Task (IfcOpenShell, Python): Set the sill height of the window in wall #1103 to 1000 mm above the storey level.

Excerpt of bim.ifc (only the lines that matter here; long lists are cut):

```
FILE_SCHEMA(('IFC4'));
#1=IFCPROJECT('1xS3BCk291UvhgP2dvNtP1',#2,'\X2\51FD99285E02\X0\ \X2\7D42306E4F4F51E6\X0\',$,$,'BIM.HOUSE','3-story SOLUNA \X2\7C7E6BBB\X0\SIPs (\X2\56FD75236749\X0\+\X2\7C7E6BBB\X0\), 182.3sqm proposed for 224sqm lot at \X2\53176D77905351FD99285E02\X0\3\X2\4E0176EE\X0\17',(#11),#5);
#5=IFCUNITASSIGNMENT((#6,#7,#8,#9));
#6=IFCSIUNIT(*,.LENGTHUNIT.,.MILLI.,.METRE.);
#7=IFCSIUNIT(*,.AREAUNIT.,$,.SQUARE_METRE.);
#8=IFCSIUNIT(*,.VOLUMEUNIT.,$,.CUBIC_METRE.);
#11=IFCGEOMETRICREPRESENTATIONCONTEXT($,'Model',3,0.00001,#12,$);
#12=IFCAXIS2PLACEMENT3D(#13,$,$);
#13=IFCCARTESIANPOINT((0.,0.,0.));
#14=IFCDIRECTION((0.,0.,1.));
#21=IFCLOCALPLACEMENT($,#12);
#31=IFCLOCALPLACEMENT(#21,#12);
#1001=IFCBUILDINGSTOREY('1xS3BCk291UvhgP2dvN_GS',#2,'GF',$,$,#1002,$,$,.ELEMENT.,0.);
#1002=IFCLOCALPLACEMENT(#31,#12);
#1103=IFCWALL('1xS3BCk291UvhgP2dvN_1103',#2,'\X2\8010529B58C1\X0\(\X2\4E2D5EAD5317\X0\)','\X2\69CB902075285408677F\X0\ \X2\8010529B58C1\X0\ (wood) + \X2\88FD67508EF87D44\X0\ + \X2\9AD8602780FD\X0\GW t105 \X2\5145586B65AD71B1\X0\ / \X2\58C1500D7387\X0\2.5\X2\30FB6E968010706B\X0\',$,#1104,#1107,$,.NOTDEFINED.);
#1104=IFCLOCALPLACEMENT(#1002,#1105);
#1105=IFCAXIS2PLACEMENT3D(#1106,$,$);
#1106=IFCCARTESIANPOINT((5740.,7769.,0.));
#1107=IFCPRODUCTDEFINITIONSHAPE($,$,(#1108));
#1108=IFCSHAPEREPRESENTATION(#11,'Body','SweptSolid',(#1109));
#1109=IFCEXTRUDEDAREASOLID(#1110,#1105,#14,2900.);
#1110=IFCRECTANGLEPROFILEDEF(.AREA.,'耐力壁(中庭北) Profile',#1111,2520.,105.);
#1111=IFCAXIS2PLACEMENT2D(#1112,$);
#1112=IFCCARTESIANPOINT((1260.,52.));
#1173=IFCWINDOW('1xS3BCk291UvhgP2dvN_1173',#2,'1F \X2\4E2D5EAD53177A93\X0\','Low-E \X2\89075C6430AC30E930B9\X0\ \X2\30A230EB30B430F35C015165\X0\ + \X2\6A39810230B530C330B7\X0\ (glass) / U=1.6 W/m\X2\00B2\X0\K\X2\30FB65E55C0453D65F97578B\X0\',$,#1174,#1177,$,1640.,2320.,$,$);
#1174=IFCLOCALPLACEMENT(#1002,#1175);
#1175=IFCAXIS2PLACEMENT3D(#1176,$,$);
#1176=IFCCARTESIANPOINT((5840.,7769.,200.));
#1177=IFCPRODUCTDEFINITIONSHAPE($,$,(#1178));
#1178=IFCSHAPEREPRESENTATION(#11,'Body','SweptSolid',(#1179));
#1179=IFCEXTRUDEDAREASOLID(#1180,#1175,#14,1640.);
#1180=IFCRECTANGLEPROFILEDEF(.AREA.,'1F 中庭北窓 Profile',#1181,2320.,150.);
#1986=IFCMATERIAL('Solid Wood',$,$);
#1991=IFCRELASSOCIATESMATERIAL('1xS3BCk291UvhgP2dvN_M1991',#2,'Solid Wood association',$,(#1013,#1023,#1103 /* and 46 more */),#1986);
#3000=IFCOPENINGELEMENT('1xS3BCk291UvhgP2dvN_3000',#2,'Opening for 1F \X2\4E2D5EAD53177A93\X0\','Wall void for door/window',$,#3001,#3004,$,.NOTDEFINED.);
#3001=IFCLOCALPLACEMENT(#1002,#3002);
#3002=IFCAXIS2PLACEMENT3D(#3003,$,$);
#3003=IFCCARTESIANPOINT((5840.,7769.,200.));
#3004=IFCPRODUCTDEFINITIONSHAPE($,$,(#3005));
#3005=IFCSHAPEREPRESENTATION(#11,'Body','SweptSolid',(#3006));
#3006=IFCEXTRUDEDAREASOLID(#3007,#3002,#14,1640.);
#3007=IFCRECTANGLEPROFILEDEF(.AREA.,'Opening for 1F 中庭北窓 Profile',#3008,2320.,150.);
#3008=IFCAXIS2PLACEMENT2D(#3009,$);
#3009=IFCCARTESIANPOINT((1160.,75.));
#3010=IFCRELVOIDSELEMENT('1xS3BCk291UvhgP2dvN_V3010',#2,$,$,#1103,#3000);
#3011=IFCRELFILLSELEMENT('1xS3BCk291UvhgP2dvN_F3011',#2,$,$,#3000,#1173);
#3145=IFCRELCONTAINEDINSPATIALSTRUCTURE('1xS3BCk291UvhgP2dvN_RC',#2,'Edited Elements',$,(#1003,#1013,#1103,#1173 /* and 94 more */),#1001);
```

```python
import numpy as np
import ifcopenshell
import ifcopenshell.api.geometry
import ifcopenshell.geom
import ifcopenshell.util.element
import ifcopenshell.util.placement
import ifcopenshell.util.shape
import ifcopenshell.util.unit

model = ifcopenshell.open("bim.ifc")
unit_scale = ifcopenshell.util.unit.calculate_unit_scale(model)

window = model.by_guid("1xS3BCk291UvhgP2dvN_1173")
opening = window.FillsVoids[0].RelatingOpeningElement
storey = ifcopenshell.util.element.get_container(window, ifc_class="IfcBuildingStorey")
level = ifcopenshell.util.placement.get_local_placement(storey.ObjectPlacement)[2, 3]

# The opening's origin need not be at the sill, so measure its lowest point.
shape = ifcopenshell.geom.create_shape(ifcopenshell.geom.settings(), opening)
bottom = ifcopenshell.util.shape.get_shape_bottom_elevation(shape, shape.geometry) / unit_scale
dz = level + 1 / unit_scale - bottom

shift = np.array([0.0, 0.0, dz])
# The window is not placed relative to its opening, so move both.
for product in (opening, window):
    matrix = ifcopenshell.util.placement.get_local_placement(product.ObjectPlacement)
    matrix[:3, 3] += shift
    ifcopenshell.api.geometry.edit_object_placement(model, product=product, matrix=matrix, is_si=False)

print(f"moved by {dz * unit_scale:+.3f} m")

model.write("bim_edited.ifc")
```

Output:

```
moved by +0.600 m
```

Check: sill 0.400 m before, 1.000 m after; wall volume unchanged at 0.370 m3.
